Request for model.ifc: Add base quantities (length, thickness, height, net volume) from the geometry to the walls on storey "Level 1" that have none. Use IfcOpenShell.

First a look at what the model holds.

```python
import ifcopenshell
import ifcopenshell.util.element
import ifcopenshell.util.unit

model = ifcopenshell.open("model.ifc")
print(model.schema)
for unit_type in ("LENGTHUNIT", "AREAUNIT", "VOLUMEUNIT"):
    print(unit_type, ifcopenshell.util.unit.calculate_unit_scale(model, unit_type))
storey = next(s for s in model.by_type("IfcBuildingStorey") if s.Name == "Level 1")
walls = [e for e in ifcopenshell.util.element.get_decomposition(storey) if e.is_a("IfcWall")]
for e in sorted(walls, key=lambda e: e.id()):
    print(e.id(), e.is_a(), e.Name, list(ifcopenshell.util.element.get_psets(e, qtos_only=True)), sep=" | ")
```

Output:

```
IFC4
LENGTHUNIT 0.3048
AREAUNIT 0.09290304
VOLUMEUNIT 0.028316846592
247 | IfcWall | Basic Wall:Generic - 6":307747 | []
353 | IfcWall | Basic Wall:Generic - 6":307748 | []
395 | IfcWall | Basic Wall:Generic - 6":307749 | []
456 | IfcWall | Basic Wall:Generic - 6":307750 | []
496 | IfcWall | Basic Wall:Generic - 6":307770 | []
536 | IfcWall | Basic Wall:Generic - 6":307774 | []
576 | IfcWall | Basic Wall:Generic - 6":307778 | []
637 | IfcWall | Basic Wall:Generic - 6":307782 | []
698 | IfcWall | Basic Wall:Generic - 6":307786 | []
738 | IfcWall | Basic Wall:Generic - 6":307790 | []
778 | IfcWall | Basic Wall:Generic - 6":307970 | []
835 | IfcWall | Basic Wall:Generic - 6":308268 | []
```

```python
import ifcopenshell
import ifcopenshell.api.pset
import ifcopenshell.geom
import ifcopenshell.util.element
import ifcopenshell.util.shape
import ifcopenshell.util.unit

model = ifcopenshell.open("model.ifc")
unit_scale = ifcopenshell.util.unit.calculate_unit_scale(model)
volume_scale = ifcopenshell.util.unit.calculate_unit_scale(model, "VOLUMEUNIT")
settings = ifcopenshell.geom.settings()

storey = next(s for s in model.by_type("IfcBuildingStorey") if s.Name == "Level 1")
walls = [e for e in ifcopenshell.util.element.get_decomposition(storey) if e.is_a("IfcWall")]

for e in sorted(walls, key=lambda e: e.id()):
    if ifcopenshell.util.element.get_psets(e, qtos_only=True, should_inherit=False):
        continue
    # Geometry comes back in metres, in the element's own axes.
    shape = ifcopenshell.geom.create_shape(settings, e)
    values = {
        "Length": ifcopenshell.util.shape.get_x(shape.geometry) / unit_scale,
        "Width": ifcopenshell.util.shape.get_y(shape.geometry) / unit_scale,
        "Height": ifcopenshell.util.shape.get_z(shape.geometry) / unit_scale,
        "NetVolume": ifcopenshell.util.shape.get_volume(shape.geometry) / volume_scale,
    }
    qto = ifcopenshell.api.pset.add_qto(model, product=e, name="Qto_WallBaseQuantities")
    ifcopenshell.api.pset.edit_qto(model, qto=qto, properties=values)
    print(e.id(), {k: round(v, 3) for k, v in values.items()})

model.write("model-out.ifc")
```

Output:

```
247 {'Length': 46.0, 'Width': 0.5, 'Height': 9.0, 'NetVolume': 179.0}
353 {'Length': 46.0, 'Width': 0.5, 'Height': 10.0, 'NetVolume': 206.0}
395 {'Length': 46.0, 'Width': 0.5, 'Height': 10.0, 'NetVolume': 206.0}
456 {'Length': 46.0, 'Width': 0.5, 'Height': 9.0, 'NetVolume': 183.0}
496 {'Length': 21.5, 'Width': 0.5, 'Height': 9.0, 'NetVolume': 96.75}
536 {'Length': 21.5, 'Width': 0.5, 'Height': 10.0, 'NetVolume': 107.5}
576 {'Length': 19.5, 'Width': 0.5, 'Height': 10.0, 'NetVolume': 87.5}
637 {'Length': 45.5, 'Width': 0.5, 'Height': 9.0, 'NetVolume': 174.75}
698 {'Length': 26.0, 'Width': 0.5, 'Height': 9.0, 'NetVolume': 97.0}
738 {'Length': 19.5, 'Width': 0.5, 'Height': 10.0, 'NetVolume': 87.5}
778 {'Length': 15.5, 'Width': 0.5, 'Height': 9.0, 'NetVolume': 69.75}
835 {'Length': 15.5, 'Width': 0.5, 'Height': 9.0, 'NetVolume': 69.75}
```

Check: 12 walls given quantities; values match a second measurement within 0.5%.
